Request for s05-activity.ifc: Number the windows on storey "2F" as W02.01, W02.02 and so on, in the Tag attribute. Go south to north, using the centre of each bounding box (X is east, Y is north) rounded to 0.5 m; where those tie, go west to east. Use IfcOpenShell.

First a look at what the model holds.

```python
import ifcopenshell
import ifcopenshell.util.element
import ifcopenshell.util.placement

model = ifcopenshell.open("s05-activity.ifc")
print(model.schema)
storey = next(s for s in model.by_type("IfcBuildingStorey") if s.Name == "2F")
windows = [e for e in ifcopenshell.util.element.get_decomposition(storey) if e.is_a("IfcWindow")]
for e in sorted(windows, key=lambda e: e.id()):
    origin = ifcopenshell.util.placement.get_local_placement(e.ObjectPlacement)[:3, 3]
    print(e.id(), e.Tag, e.Name, origin.round(2) + 0.0, sep=" | ")
```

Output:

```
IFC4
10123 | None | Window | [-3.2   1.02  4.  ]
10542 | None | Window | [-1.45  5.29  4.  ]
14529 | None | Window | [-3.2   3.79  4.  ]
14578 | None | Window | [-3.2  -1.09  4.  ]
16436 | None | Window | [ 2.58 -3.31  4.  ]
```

```python
import ifcopenshell
import ifcopenshell.geom
import ifcopenshell.util.element
import ifcopenshell.util.shape

model = ifcopenshell.open("s05-activity.ifc")
settings = ifcopenshell.geom.settings()
settings.set("use-world-coords", True)


def centre(element):
    shape = ifcopenshell.geom.create_shape(settings, element)
    return ifcopenshell.util.shape.get_bbox_centroid(shape.geometry)


storey = next(s for s in model.by_type("IfcBuildingStorey") if s.Name == "2F")
windows = [e for e in ifcopenshell.util.element.get_decomposition(storey) if e.is_a("IfcWindow")]

# Insertion points can sit at a corner or the storey origin, so sort by the geometry (in metres).
centres = {e: centre(e) for e in windows}
windows.sort(key=lambda e: (round(centres[e][1] / 0.5), centres[e][0]))

for i, e in enumerate(windows, start=1):
    number = f"W02.{i:02d}"
    e.Tag = number
    print(e.id(), number)

model.write("s05-activity-out.ifc")
```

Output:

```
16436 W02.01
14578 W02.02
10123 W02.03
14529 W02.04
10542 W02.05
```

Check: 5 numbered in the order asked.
